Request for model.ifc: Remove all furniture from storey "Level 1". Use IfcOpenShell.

First a look at what the model holds.

```python
import ifcopenshell
import ifcopenshell.util.element

model = ifcopenshell.open("model.ifc")
print(model.schema)
storey = next(s for s in model.by_type("IfcBuildingStorey") if s.Name == "Level 1")
furniture = [e for e in ifcopenshell.util.element.get_decomposition(storey) if e.is_a("IfcFurnishingElement")]
seen = {}
for e in furniture:
    element_type = ifcopenshell.util.element.get_type(e)
    name = element_type.Name if element_type not in (None, e) else None
    seen[name] = seen.get(name, 0) + 1
for name, count in sorted(seen.items(), key=str):
    print(count, "x", name)
```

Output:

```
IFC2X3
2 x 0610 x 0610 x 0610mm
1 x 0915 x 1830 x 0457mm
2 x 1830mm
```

```python
import ifcopenshell
import ifcopenshell.api.root
import ifcopenshell.util.element

model = ifcopenshell.open("model.ifc")

storey = next(s for s in model.by_type("IfcBuildingStorey") if s.Name == "Level 1")
furniture = [e for e in ifcopenshell.util.element.get_decomposition(storey) if e.is_a("IfcFurnishingElement")]

for e in furniture:
    ifcopenshell.api.root.remove_product(model, product=e)
print(len(furniture), "removed")

model.write("model_updated.ifc")
```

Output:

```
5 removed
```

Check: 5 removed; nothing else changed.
